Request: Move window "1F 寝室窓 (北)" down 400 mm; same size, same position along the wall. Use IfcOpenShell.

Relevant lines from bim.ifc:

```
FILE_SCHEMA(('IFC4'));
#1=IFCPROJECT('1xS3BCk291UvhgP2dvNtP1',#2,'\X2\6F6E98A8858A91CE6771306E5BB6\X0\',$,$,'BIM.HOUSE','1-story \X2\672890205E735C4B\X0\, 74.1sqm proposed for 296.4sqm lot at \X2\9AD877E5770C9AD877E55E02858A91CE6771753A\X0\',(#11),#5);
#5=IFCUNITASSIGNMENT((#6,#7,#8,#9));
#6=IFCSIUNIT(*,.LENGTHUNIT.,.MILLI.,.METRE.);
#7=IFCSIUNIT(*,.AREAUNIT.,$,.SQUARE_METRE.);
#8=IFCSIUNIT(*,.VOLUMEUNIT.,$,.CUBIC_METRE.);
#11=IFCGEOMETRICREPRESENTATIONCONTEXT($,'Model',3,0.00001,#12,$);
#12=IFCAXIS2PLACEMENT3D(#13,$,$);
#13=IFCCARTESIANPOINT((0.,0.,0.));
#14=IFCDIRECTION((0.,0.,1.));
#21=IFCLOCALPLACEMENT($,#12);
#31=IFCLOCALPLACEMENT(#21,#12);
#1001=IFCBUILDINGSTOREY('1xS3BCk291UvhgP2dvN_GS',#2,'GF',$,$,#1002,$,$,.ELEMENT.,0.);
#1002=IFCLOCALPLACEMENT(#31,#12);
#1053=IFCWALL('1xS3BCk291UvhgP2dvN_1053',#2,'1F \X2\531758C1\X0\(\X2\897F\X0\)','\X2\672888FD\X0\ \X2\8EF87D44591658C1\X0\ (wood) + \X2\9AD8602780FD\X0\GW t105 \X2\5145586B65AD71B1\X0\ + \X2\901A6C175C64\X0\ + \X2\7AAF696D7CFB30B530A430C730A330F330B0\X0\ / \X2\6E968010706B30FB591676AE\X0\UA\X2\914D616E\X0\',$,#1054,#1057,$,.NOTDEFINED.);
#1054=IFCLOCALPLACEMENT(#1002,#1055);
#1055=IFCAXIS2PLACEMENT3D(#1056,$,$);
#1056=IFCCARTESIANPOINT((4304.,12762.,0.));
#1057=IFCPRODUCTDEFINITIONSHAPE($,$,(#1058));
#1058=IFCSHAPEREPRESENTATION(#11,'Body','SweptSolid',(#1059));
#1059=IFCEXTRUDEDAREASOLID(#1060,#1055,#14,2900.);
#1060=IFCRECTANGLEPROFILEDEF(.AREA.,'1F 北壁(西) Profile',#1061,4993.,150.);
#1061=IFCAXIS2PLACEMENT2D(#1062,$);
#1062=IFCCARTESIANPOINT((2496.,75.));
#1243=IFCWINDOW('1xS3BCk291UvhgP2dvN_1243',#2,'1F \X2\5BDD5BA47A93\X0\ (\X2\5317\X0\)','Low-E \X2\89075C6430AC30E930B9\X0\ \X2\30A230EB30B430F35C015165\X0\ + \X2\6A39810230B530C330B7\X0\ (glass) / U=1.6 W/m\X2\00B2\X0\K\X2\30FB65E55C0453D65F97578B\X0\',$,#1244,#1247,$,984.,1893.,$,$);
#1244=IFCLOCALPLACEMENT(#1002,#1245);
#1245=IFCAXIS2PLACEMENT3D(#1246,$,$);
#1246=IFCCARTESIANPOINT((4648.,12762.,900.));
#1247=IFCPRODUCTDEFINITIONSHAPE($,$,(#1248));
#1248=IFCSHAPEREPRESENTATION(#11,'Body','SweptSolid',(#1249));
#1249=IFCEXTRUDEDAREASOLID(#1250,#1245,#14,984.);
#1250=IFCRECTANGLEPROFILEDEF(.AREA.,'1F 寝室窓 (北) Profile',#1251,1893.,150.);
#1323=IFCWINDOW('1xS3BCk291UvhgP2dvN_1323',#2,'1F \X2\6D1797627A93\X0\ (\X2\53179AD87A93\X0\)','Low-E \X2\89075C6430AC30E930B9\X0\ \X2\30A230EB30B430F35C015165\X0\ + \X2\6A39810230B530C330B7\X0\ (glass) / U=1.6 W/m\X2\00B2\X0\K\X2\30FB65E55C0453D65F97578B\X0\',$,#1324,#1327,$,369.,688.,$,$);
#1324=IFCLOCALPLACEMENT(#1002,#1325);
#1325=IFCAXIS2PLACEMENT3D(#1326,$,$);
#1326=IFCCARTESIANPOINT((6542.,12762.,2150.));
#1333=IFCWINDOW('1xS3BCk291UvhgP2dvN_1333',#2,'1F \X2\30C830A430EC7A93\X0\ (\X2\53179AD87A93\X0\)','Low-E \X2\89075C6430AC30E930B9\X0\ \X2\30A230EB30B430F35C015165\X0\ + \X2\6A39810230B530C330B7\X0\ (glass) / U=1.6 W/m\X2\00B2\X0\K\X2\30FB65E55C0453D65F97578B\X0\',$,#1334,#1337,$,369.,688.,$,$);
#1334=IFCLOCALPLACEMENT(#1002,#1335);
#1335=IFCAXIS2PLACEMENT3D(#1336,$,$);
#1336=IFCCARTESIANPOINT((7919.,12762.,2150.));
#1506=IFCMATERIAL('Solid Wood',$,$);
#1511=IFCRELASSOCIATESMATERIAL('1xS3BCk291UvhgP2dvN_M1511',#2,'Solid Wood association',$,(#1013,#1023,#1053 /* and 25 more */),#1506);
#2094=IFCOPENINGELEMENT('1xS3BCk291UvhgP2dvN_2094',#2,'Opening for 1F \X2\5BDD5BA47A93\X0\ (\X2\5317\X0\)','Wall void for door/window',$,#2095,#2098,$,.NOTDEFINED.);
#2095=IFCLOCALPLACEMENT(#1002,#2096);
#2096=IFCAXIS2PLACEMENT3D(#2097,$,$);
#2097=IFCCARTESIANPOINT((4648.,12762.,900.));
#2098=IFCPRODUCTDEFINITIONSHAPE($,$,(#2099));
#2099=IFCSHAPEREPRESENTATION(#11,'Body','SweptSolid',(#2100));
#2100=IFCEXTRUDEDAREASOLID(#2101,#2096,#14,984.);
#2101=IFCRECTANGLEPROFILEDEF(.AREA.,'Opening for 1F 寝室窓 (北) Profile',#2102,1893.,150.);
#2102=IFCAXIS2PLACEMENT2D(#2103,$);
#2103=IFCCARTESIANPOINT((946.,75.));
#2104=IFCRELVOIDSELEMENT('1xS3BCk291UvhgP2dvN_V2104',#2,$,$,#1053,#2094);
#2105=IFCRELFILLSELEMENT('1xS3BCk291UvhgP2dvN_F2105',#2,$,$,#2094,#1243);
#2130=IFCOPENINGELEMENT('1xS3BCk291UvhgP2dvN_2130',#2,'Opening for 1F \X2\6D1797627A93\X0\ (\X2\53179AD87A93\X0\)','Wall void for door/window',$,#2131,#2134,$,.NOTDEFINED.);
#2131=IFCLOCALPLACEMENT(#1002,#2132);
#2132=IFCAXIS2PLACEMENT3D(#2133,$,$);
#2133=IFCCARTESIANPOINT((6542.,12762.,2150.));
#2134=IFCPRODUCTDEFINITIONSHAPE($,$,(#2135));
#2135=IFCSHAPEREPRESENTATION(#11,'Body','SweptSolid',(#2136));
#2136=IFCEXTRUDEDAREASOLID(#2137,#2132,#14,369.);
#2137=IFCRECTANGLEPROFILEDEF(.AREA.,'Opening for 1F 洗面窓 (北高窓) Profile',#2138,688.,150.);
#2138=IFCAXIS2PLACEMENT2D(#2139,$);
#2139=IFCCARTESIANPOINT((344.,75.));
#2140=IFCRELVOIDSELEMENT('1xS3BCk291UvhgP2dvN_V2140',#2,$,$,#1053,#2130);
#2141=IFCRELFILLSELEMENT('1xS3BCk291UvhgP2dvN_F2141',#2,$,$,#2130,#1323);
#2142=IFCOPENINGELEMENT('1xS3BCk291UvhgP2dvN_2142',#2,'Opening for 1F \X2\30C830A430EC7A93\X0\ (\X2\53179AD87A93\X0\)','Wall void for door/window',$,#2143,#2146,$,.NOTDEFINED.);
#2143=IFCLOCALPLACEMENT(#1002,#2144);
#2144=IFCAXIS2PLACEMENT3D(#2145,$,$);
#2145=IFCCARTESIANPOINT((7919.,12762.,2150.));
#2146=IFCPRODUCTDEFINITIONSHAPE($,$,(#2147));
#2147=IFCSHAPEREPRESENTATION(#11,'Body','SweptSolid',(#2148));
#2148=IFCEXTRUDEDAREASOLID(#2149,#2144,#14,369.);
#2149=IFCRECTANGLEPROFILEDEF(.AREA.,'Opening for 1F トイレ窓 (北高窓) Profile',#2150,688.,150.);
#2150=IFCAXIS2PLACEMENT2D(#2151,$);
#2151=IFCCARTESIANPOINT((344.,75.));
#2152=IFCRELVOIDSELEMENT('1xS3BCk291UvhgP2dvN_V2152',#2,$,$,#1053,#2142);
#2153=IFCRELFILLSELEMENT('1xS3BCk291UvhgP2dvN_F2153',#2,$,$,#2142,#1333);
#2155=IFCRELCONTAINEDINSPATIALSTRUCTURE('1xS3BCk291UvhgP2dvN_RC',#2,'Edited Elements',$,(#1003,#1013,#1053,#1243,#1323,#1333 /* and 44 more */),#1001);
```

```python
import numpy as np
import ifcopenshell
import ifcopenshell.api.geometry
import ifcopenshell.util.placement
import ifcopenshell.util.unit

model = ifcopenshell.open("bim.ifc")
unit_scale = ifcopenshell.util.unit.calculate_unit_scale(model)

window = model.by_guid("1xS3BCk291UvhgP2dvN_1243")
opening = window.FillsVoids[0].RelatingOpeningElement
dz = -0.4 / unit_scale

shift = np.array([0.0, 0.0, dz])
# The window is not placed relative to its opening, so move both.
for product in (opening, window):
    matrix = ifcopenshell.util.placement.get_local_placement(product.ObjectPlacement)
    matrix[:3, 3] += shift
    ifcopenshell.api.geometry.edit_object_placement(model, product=product, matrix=matrix, is_si=False)

print(f"moved by {dz * unit_scale:+.3f} m")

model.write("bim_rev.ifc")
```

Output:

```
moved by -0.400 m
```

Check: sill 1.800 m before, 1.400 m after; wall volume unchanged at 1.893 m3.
